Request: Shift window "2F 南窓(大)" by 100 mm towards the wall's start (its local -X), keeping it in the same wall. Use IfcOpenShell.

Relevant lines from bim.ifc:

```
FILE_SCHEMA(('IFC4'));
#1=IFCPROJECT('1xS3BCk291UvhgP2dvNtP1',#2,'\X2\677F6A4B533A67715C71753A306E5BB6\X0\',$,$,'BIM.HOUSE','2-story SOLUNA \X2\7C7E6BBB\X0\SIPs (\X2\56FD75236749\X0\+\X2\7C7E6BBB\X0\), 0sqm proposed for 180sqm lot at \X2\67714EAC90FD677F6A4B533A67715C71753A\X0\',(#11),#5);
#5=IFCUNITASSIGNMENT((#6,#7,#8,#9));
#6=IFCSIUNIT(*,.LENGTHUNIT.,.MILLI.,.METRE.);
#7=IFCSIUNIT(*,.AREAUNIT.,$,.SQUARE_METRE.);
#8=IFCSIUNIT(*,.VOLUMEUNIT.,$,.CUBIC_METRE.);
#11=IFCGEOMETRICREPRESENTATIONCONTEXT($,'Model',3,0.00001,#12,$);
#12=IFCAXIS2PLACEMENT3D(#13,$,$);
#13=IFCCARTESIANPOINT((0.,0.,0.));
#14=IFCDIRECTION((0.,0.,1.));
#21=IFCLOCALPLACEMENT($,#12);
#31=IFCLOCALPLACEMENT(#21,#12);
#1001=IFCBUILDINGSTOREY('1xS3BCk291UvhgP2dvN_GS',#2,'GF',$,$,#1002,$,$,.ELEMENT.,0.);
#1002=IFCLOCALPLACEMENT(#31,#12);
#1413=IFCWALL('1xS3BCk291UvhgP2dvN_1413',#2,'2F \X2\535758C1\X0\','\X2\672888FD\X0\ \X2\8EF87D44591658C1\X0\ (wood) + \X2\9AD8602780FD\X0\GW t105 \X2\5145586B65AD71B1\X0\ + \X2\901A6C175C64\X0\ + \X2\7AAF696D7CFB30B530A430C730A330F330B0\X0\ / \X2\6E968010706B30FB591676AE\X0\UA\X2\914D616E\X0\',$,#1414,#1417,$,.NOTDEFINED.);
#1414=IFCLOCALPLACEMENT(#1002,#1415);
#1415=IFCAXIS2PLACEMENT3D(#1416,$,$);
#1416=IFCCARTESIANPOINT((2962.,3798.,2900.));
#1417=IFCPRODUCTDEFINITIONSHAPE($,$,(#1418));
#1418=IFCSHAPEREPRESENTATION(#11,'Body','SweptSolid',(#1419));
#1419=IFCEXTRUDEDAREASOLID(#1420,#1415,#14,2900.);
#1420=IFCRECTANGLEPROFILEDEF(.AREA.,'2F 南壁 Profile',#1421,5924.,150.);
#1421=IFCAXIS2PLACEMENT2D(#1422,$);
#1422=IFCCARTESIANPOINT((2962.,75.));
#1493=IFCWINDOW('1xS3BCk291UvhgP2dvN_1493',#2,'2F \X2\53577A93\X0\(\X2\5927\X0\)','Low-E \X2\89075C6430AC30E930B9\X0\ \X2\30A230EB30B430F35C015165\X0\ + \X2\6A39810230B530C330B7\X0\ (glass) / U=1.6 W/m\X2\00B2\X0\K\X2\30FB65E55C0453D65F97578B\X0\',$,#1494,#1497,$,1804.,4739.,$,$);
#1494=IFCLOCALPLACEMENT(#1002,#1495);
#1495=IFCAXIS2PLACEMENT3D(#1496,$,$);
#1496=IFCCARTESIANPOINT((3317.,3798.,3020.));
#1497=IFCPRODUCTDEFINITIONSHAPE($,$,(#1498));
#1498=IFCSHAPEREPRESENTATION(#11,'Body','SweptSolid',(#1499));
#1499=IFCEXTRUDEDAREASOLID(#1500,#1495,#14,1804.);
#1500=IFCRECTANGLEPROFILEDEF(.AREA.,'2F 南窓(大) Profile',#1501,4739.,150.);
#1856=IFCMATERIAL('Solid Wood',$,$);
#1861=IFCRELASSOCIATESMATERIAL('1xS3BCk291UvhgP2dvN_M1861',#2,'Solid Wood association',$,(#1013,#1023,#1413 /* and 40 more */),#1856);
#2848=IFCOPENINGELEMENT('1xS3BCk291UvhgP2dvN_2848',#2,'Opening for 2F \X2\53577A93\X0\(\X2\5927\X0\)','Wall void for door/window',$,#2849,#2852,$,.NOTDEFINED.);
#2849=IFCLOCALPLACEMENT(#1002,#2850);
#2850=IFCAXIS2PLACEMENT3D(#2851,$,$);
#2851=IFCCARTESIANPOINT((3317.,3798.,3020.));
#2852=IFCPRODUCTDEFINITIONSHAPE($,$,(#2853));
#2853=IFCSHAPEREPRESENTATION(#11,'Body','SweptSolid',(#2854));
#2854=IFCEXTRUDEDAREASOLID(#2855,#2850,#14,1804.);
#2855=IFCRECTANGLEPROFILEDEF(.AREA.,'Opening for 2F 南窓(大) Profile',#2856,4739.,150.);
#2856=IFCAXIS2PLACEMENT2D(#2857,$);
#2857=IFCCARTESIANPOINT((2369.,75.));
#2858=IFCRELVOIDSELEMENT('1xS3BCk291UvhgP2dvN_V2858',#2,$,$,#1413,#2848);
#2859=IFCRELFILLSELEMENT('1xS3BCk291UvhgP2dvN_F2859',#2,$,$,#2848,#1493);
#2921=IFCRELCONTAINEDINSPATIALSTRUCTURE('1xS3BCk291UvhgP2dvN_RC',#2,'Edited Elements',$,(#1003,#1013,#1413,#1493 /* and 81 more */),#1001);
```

```python
import ifcopenshell
import ifcopenshell.api.geometry
import ifcopenshell.util.placement

model = ifcopenshell.open("bim.ifc")

window = model.by_guid("1xS3BCk291UvhgP2dvN_1493")
opening = window.FillsVoids[0].RelatingOpeningElement
wall = opening.VoidsElements[0].RelatingBuildingElement

wall_matrix = ifcopenshell.util.placement.get_local_placement(wall.ObjectPlacement)
shift = wall_matrix[:3, 0] * -100.0
before = ifcopenshell.util.placement.get_local_placement(window.ObjectPlacement)[:3, 3].copy()

# The window is not placed relative to its opening, so move both.
for product in (opening, window):
    matrix = ifcopenshell.util.placement.get_local_placement(product.ObjectPlacement)
    matrix[:3, 3] += shift
    ifcopenshell.api.geometry.edit_object_placement(model, product=product, matrix=matrix, is_si=False)

after = ifcopenshell.util.placement.get_local_placement(window.ObjectPlacement)[:3, 3]
print("window moved by", (after - before).round(3) + 0.0)

model.write("bim_updated.ifc")
```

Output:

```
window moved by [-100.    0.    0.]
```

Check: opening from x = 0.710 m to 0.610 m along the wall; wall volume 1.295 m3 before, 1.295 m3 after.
